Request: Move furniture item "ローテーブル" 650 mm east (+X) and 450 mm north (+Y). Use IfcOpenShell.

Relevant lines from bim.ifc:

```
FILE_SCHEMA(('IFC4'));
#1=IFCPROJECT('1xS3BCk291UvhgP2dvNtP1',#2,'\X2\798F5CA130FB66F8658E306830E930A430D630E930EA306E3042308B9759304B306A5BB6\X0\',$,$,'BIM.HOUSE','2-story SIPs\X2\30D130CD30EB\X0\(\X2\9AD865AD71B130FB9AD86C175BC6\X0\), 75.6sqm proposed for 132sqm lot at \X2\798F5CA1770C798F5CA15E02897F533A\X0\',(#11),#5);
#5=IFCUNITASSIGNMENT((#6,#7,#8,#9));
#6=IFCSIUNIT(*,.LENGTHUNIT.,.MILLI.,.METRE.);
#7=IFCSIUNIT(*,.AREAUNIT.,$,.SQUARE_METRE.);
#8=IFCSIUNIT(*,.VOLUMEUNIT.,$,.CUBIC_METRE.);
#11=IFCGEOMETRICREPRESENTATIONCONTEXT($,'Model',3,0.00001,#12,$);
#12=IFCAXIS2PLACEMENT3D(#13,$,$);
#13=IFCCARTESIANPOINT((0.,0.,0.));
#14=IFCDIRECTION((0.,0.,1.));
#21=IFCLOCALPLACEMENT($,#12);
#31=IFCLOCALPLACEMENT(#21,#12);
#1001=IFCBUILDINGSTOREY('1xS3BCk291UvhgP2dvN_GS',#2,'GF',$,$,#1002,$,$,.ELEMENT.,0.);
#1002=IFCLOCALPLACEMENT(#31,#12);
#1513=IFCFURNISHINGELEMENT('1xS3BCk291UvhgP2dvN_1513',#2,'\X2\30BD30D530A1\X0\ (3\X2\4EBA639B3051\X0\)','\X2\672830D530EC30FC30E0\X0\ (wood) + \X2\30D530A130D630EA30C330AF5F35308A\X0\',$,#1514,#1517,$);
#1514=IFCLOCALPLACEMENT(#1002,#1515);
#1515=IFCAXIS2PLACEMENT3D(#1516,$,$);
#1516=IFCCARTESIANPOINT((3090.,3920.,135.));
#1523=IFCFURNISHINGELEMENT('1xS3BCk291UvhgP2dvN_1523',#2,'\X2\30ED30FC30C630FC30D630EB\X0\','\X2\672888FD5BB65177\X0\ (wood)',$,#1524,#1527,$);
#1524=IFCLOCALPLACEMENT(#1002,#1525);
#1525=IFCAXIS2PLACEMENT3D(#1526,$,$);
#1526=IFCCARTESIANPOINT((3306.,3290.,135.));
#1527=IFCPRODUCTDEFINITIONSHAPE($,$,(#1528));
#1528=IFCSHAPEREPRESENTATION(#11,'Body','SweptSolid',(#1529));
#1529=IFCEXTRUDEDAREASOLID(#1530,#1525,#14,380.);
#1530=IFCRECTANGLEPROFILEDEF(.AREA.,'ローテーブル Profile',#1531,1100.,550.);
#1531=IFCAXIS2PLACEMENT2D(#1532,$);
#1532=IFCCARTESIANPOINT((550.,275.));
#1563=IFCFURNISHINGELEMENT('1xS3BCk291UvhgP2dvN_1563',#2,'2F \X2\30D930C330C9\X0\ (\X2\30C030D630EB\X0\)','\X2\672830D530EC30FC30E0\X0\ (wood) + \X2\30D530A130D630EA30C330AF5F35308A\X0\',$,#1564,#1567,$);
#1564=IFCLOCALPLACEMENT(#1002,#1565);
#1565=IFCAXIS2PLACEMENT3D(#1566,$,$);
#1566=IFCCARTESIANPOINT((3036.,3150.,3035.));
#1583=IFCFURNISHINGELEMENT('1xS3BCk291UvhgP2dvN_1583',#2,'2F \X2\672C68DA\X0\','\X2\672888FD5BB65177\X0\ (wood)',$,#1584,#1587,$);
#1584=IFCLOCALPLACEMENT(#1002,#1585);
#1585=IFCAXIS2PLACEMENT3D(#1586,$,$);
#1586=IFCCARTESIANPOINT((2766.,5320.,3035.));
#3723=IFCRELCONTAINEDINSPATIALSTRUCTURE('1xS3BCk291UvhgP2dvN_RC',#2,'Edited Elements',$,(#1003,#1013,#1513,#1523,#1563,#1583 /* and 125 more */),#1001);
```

```python
import ifcopenshell
import ifcopenshell.api.geometry
import ifcopenshell.util.placement

model = ifcopenshell.open("bim.ifc")

item = model.by_guid("1xS3BCk291UvhgP2dvN_1523")
matrix = ifcopenshell.util.placement.get_local_placement(item.ObjectPlacement)
matrix[0, 3] += 650.0
matrix[1, 3] += 450.0
ifcopenshell.api.geometry.edit_object_placement(model, product=item, matrix=matrix, is_si=False)

print(ifcopenshell.util.placement.get_local_placement(item.ObjectPlacement).round(3) + 0.0)

model.write("bim-out.ifc")
```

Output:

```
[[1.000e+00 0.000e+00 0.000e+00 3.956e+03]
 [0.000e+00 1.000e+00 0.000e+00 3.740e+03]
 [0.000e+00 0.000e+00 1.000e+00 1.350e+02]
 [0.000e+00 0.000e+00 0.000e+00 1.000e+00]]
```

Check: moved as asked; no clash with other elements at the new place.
